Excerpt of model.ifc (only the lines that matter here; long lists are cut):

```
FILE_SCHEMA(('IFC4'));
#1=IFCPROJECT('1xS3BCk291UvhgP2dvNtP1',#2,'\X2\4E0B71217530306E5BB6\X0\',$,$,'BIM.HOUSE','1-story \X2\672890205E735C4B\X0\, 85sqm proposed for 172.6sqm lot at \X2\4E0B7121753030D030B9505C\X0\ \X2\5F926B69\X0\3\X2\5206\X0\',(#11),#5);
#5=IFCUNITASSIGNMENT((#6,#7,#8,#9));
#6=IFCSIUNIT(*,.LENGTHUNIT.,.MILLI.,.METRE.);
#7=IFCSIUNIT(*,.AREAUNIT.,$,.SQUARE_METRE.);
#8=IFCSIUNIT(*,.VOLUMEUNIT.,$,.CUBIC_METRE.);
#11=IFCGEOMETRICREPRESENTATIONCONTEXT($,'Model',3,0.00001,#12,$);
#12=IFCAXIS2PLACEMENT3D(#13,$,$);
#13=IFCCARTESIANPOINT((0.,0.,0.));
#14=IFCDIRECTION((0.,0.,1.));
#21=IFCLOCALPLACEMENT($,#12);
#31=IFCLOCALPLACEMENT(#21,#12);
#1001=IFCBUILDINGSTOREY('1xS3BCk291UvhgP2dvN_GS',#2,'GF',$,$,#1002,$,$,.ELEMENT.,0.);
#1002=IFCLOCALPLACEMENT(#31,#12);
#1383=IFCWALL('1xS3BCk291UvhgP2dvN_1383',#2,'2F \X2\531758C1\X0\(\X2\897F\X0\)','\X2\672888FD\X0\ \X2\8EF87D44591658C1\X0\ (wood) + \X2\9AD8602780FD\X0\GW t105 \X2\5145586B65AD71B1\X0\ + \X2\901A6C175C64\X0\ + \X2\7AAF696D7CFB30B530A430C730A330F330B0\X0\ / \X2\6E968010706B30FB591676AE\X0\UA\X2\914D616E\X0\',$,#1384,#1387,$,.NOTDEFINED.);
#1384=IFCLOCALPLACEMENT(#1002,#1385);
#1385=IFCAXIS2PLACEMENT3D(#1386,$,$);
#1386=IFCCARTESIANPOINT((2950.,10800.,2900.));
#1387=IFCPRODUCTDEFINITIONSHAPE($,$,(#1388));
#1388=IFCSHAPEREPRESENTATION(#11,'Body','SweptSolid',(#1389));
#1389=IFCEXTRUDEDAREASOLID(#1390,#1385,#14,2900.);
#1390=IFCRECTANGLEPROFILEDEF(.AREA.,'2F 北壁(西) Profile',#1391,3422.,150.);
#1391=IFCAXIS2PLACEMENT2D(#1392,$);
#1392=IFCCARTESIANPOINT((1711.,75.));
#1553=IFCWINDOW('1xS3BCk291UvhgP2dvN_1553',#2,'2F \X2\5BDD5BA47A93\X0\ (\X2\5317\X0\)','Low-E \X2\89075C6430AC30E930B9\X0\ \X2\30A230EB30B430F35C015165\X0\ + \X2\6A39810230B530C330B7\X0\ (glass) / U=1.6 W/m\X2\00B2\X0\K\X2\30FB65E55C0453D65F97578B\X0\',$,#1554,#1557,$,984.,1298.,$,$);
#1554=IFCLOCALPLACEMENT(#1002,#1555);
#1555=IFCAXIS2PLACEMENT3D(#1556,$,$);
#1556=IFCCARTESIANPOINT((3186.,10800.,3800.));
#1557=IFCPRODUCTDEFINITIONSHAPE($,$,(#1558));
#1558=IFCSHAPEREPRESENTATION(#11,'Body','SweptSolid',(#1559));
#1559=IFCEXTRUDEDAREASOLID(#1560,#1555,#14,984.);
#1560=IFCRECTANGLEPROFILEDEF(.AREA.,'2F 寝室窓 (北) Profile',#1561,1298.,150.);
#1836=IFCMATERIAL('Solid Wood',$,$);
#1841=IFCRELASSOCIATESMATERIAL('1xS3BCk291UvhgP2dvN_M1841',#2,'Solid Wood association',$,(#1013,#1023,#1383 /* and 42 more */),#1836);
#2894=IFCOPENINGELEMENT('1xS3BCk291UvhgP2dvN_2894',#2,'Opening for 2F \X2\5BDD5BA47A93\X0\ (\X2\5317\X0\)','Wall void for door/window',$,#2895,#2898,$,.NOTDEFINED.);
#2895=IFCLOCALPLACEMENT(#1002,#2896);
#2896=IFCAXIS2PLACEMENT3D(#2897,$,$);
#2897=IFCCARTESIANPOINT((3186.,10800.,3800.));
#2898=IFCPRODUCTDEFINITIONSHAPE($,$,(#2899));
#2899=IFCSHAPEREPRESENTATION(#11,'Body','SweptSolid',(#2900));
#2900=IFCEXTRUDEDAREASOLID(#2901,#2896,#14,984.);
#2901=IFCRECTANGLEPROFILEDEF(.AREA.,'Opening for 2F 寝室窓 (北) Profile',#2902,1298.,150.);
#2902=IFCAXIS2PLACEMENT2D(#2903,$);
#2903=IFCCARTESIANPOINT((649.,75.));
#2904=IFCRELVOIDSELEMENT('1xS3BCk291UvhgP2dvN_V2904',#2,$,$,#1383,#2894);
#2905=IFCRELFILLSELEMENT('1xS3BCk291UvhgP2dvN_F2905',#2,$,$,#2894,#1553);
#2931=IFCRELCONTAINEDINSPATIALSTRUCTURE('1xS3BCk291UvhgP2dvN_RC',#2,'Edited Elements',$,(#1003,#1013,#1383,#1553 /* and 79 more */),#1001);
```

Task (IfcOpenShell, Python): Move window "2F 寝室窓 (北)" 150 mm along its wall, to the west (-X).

```python
import ifcopenshell
import ifcopenshell.api.geometry
import ifcopenshell.util.placement

model = ifcopenshell.open("model.ifc")

window = model.by_guid("1xS3BCk291UvhgP2dvN_1553")
opening = window.FillsVoids[0].RelatingOpeningElement
wall = opening.VoidsElements[0].RelatingBuildingElement

wall_matrix = ifcopenshell.util.placement.get_local_placement(wall.ObjectPlacement)
shift = wall_matrix[:3, 0] * -150.0
before = ifcopenshell.util.placement.get_local_placement(window.ObjectPlacement)[:3, 3].copy()

# The window is not placed relative to its opening, so move both.
for product in (opening, window):
    matrix = ifcopenshell.util.placement.get_local_placement(product.ObjectPlacement)
    matrix[:3, 3] += shift
    ifcopenshell.api.geometry.edit_object_placement(model, product=product, matrix=matrix, is_si=False)

after = ifcopenshell.util.placement.get_local_placement(window.ObjectPlacement)[:3, 3]
print("window moved by", (after - before).round(3) + 0.0)

model.write("model-out.ifc")
```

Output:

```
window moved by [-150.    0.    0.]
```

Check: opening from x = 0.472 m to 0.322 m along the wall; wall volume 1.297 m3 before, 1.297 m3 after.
